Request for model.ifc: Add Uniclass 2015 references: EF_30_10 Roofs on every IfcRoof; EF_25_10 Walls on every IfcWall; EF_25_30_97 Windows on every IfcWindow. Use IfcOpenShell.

First a look at what the model holds.

```python
import ifcopenshell

model = ifcopenshell.open("model.ifc")
print(model.schema)
print("classifications:", [c.Name for c in model.by_type("IfcClassification")])
for ifc_class in ("IfcDoor", "IfcRoof", "IfcStair", "IfcWall", "IfcWindow"):
    print(ifc_class, len(model.by_type(ifc_class)))
```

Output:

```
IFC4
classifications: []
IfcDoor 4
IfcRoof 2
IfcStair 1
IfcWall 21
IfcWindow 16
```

```python
import ifcopenshell
import ifcopenshell.api.classification

model = ifcopenshell.open("model.ifc")

system = ifcopenshell.api.classification.add_classification(model, classification="Uniclass 2015")

codes = {
    "IfcRoof": ("EF_30_10", "Roofs"),
    "IfcWall": ("EF_25_10", "Walls"),
    "IfcWindow": ("EF_25_30_97", "Windows"),
}
for ifc_class, (code, name) in codes.items():
    products = model.by_type(ifc_class)
    ifcopenshell.api.classification.add_reference(
        model, products=products, classification=system, identification=code, name=name
    )
    print(code, len(products))

model.write("model-out.ifc")
```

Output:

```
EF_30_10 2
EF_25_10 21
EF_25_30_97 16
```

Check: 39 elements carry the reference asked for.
